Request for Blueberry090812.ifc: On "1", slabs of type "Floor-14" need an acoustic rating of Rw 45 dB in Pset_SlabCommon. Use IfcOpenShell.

First a look at what the model holds.

```python
import ifcopenshell
import ifcopenshell.util.element

model = ifcopenshell.open("Blueberry090812.ifc")
print(model.schema)
storey = next(s for s in model.by_type("IfcBuildingStorey") if s.Name == "1")
slabs = [e for e in ifcopenshell.util.element.get_decomposition(storey) if e.is_a("IfcSlab")]
seen = {}
for e in slabs:
    element_type = ifcopenshell.util.element.get_type(e)
    key = (element_type.Name if element_type != e and element_type else None, ifcopenshell.util.element.get_pset(e, "Pset_SlabCommon", "AcousticRating"))
    seen[key] = seen.get(key, 0) + 1
for (name, value), count in sorted(seen.items(), key=str):
    print(count, "x", name, "|", value)
```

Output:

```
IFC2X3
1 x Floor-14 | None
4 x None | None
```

```python
import ifcopenshell
import ifcopenshell.api.pset
import ifcopenshell.util.element

model = ifcopenshell.open("Blueberry090812.ifc")

storey = next(s for s in model.by_type("IfcBuildingStorey") if s.Name == "1")
slabs = [e for e in ifcopenshell.util.element.get_decomposition(storey) if e.is_a("IfcSlab")]

count = 0
for e in slabs:
    element_type = ifcopenshell.util.element.get_type(e)
    if element_type in (None, e) or element_type.Name != "Floor-14":
        continue
    found = ifcopenshell.util.element.get_pset(e, "Pset_SlabCommon", should_inherit=False)
    if found:
        pset = model.by_id(found["id"])
        if len(ifcopenshell.util.element.get_elements_by_pset(pset)) > 1:
            pset = ifcopenshell.api.pset.unshare_pset(model, products=[e], pset=pset)[0]
    else:
        pset = ifcopenshell.api.pset.add_pset(model, product=e, name="Pset_SlabCommon")
    ifcopenshell.api.pset.edit_pset(model, pset=pset, properties={"AcousticRating": "Rw 45 dB"})
    count += 1

print(count, "slabs updated")

model.write("Blueberry090812_rev.ifc")
```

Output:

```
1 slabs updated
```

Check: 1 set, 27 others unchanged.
